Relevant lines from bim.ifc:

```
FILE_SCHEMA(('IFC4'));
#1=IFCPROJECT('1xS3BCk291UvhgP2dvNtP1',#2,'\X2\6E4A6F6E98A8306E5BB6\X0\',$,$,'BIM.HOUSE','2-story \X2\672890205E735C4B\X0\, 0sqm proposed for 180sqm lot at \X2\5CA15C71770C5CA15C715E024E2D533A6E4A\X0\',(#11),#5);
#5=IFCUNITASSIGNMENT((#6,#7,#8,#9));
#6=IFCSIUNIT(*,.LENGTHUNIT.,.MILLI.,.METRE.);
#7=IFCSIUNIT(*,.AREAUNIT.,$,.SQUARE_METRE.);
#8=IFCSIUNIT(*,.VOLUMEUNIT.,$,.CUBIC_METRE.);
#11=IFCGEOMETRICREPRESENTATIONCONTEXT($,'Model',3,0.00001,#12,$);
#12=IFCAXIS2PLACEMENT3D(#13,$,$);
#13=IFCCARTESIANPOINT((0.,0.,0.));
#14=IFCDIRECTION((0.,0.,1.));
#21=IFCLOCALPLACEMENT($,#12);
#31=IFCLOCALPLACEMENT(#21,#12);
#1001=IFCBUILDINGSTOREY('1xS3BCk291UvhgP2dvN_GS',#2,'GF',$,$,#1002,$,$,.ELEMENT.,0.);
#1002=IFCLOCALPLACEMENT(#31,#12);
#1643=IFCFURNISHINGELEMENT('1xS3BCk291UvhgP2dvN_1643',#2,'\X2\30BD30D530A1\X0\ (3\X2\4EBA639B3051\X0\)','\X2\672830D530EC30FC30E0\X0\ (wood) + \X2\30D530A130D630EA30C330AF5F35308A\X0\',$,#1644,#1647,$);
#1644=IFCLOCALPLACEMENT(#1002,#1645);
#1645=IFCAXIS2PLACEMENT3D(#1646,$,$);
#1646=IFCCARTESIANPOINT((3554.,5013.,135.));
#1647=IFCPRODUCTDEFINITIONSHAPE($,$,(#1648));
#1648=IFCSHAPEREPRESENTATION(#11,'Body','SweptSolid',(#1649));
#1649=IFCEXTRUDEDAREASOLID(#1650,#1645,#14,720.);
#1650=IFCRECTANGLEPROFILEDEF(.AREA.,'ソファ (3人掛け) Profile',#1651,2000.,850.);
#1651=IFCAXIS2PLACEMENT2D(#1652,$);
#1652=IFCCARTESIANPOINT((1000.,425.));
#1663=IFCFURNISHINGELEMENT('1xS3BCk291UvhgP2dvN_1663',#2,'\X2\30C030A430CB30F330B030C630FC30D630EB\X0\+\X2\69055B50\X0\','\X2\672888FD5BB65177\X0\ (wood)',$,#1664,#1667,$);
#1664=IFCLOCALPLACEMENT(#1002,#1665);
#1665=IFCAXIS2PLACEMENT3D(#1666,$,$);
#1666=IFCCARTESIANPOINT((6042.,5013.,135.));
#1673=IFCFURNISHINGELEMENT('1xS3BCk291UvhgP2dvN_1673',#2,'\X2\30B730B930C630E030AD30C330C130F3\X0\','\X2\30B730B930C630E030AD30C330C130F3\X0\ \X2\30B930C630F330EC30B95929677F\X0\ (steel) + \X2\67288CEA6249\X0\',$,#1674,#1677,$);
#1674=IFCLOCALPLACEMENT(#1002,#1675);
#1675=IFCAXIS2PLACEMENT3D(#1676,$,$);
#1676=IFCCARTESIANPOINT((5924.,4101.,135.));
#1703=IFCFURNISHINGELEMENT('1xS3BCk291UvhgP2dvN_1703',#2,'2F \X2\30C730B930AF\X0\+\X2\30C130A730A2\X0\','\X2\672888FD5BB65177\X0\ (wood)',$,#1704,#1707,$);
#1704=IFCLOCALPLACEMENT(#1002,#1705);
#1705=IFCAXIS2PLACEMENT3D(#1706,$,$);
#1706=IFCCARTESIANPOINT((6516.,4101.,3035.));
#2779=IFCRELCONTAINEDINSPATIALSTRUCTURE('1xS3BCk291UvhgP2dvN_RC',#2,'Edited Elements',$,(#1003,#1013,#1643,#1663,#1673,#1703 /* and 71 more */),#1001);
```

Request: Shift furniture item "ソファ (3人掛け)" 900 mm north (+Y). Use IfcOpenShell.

```python
import ifcopenshell
import ifcopenshell.api.geometry
import ifcopenshell.util.placement

model = ifcopenshell.open("bim.ifc")

item = model.by_guid("1xS3BCk291UvhgP2dvN_1643")
matrix = ifcopenshell.util.placement.get_local_placement(item.ObjectPlacement)
matrix[1, 3] += 900.0
ifcopenshell.api.geometry.edit_object_placement(model, product=item, matrix=matrix, is_si=False)

print(ifcopenshell.util.placement.get_local_placement(item.ObjectPlacement).round(3) + 0.0)

model.write("bim_rev.ifc")
```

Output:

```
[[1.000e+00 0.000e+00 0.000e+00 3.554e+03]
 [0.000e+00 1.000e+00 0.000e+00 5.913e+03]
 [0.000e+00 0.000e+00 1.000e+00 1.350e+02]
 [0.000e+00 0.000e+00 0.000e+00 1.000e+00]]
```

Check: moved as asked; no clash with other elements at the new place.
